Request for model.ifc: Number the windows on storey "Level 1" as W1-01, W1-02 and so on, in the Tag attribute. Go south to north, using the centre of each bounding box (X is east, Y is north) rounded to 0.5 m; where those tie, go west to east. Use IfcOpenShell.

First a look at what the model holds.

```python
import ifcopenshell
import ifcopenshell.util.element
import ifcopenshell.util.placement

model = ifcopenshell.open("model.ifc")
print(model.schema)
storey = next(s for s in model.by_type("IfcBuildingStorey") if s.Name == "Level 1")
windows = [e for e in ifcopenshell.util.element.get_decomposition(storey) if e.is_a("IfcWindow")]
for e in sorted(windows, key=lambda e: e.id()):
    origin = ifcopenshell.util.placement.get_local_placement(e.ObjectPlacement)[:3, 3]
    print(e.id(), e.Tag, e.Name, origin.round(2) + 0.0, sep=" | ")
```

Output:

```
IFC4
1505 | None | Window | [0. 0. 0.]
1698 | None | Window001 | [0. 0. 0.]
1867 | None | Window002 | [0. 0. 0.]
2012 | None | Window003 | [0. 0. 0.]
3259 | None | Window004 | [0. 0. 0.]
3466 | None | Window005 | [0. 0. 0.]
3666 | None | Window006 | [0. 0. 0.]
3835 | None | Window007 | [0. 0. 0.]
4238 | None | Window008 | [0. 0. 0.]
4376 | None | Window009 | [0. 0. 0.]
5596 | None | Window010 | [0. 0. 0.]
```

```python
import ifcopenshell
import ifcopenshell.geom
import ifcopenshell.util.element
import ifcopenshell.util.shape

model = ifcopenshell.open("model.ifc")
settings = ifcopenshell.geom.settings()
settings.set("use-world-coords", True)


def centre(element):
    shape = ifcopenshell.geom.create_shape(settings, element)
    return ifcopenshell.util.shape.get_bbox_centroid(shape.geometry)


storey = next(s for s in model.by_type("IfcBuildingStorey") if s.Name == "Level 1")
windows = [e for e in ifcopenshell.util.element.get_decomposition(storey) if e.is_a("IfcWindow")]

# Insertion points can sit at a corner or the storey origin, so sort by the geometry (in metres).
centres = {e: centre(e) for e in windows}
windows.sort(key=lambda e: (round(centres[e][1] / 0.5), centres[e][0]))

for i, e in enumerate(windows, start=1):
    number = f"W1-{i:02d}"
    e.Tag = number
    print(e.id(), number)

model.write("model_updated.ifc")
```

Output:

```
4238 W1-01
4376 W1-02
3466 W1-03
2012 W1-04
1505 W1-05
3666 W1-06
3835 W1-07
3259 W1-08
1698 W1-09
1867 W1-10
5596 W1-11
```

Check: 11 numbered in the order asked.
